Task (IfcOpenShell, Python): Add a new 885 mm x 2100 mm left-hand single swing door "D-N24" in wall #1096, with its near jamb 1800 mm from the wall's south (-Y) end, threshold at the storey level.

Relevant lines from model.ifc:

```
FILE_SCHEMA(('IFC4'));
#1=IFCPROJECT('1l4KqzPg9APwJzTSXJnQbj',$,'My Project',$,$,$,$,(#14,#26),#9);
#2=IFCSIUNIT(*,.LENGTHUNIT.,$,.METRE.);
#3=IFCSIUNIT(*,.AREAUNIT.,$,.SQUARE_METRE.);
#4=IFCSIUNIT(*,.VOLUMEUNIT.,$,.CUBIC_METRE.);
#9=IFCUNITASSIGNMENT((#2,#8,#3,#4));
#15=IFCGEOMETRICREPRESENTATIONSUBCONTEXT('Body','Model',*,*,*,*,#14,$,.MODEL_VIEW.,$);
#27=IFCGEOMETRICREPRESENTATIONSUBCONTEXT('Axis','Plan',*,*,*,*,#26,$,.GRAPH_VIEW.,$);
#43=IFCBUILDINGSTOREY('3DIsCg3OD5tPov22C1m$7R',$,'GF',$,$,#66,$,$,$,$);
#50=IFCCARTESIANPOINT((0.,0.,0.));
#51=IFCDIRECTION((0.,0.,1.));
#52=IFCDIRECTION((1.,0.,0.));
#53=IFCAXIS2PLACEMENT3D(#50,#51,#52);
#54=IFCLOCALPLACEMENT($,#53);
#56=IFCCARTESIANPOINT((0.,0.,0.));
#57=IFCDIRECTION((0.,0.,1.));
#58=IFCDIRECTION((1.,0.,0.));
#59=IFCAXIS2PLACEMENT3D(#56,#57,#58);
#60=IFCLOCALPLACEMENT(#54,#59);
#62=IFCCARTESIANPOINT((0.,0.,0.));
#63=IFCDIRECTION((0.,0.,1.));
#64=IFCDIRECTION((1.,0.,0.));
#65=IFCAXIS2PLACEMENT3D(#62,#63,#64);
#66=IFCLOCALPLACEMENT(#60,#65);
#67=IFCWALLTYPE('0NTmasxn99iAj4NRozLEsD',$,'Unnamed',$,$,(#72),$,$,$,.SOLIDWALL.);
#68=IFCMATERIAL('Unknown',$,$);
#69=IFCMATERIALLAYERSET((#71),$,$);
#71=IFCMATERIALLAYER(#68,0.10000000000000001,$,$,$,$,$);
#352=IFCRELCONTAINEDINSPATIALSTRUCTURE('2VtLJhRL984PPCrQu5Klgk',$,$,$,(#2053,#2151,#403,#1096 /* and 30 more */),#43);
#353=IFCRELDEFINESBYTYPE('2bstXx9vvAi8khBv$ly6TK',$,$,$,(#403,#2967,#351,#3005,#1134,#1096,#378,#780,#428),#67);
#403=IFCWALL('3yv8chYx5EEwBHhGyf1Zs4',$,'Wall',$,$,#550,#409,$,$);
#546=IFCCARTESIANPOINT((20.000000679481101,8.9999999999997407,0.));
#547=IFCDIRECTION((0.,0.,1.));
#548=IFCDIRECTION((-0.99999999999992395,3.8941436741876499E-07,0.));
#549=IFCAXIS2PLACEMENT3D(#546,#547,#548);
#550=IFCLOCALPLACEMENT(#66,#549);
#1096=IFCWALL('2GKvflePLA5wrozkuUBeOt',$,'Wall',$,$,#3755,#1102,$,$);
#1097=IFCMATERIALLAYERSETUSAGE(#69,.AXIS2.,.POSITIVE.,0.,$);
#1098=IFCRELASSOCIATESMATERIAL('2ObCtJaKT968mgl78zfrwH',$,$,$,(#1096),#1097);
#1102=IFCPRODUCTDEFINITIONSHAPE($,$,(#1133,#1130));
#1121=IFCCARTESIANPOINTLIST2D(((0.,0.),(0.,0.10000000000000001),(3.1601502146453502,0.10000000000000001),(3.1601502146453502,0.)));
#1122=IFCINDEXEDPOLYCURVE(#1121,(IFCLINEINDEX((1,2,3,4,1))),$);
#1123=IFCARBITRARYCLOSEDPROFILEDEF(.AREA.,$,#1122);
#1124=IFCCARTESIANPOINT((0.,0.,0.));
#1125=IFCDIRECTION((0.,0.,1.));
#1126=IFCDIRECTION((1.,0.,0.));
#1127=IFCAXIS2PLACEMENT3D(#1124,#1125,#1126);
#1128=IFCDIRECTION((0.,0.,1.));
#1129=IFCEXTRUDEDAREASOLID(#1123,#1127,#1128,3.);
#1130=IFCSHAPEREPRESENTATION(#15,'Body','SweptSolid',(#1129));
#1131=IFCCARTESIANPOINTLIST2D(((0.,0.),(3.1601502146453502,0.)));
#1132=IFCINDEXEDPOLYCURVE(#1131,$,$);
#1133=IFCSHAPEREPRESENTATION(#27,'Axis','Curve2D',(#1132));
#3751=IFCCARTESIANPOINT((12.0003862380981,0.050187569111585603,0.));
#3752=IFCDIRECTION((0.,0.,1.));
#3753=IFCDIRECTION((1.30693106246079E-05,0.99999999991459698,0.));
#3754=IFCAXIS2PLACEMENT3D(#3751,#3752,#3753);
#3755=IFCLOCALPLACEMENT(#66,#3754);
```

```python
import numpy as np
import ifcopenshell
import ifcopenshell.api.feature
import ifcopenshell.api.geometry
import ifcopenshell.api.root
import ifcopenshell.api.spatial
import ifcopenshell.geom
import ifcopenshell.util.element
import ifcopenshell.util.placement
import ifcopenshell.util.representation
import ifcopenshell.util.shape
import ifcopenshell.util.unit

model = ifcopenshell.open("model.ifc")
unit_scale = ifcopenshell.util.unit.calculate_unit_scale(model)
settings = ifcopenshell.geom.settings()


def volume(element):
    """Net volume in cubic metres, openings subtracted."""
    shape = ifcopenshell.geom.create_shape(settings, element)
    return ifcopenshell.util.shape.get_volume(shape.geometry)


wall = model.by_guid("2GKvflePLA5wrozkuUBeOt")
storey = ifcopenshell.util.element.get_container(wall, ifc_class="IfcBuildingStorey")
context = ifcopenshell.util.representation.get_context(model, "Model", "Body", "MODEL_VIEW")
before = volume(wall)

width, height, from_end, sill = 0.885, 2.1, 1.8, 0.0  # metres

# The wall runs along its own X axis, and the end named is its -X end.
wall_shape = ifcopenshell.geom.create_shape(settings, wall)
x, y, z = ifcopenshell.util.shape.get_vertices(wall_shape.geometry).T
start = x.min() + from_end
face, thickness = float(y.min()), float(y.max() - y.min())
wall_matrix = ifcopenshell.util.placement.get_local_placement(wall.ObjectPlacement)
level = ifcopenshell.util.placement.get_local_placement(storey.ObjectPlacement)[2, 3]


def in_wall(x, y):
    """Placement at x, y metres in the wall's axes, at sill height."""
    matrix = wall_matrix.copy()
    matrix[:, 3] = wall_matrix @ np.array([x / unit_scale, y / unit_scale, 0.0, 1.0])
    matrix[2, 3] = level + sill / unit_scale
    return matrix


# Opening: a box that overshoots both wall faces by 50 mm.
opening = ifcopenshell.api.root.create_entity(model, ifc_class="IfcOpeningElement", predefined_type="OPENING")
box = ifcopenshell.api.geometry.add_wall_representation(
    model, context=context, length=width, height=height, thickness=thickness + 0.1
)
ifcopenshell.api.geometry.assign_representation(model, product=opening, representation=box)
ifcopenshell.api.geometry.edit_object_placement(model, product=opening, matrix=in_wall(start, face - 0.05), is_si=False)
ifcopenshell.api.feature.add_feature(model, feature=opening, element=wall)

door = ifcopenshell.api.root.create_entity(model, ifc_class="IfcDoor", name="D-N24", predefined_type="DOOR")
door.OverallWidth, door.OverallHeight = width / unit_scale, height / unit_scale
door.OperationType = "SINGLE_SWING_LEFT"
body = ifcopenshell.api.geometry.add_door_representation(
    model,
    context=context,
    overall_width=door.OverallWidth,
    overall_height=door.OverallHeight,
    operation_type="SINGLE_SWING_LEFT",
    lining_properties={"LiningDepth": thickness / unit_scale, "ThresholdDepth": thickness / unit_scale},
)
ifcopenshell.api.geometry.assign_representation(model, product=door, representation=body)
ifcopenshell.api.spatial.assign_container(model, products=[door], relating_structure=storey)
ifcopenshell.api.feature.add_filling(model, opening=opening, element=door)

# The lining spans the wall, so the door starts at the wall face.
ifcopenshell.api.geometry.edit_object_placement(model, product=door, matrix=in_wall(start, face), is_si=False)

after = volume(wall)

print(f"wall volume {before:.3f} -> {after:.3f} m3")

model.write("model_edited.ifc")
```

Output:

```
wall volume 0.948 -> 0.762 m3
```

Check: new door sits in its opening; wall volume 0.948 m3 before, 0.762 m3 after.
